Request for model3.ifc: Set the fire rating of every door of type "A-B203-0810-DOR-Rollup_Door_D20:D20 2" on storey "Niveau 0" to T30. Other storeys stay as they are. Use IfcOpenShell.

First a look at what the model holds.

```python
import ifcopenshell
import ifcopenshell.util.element

model = ifcopenshell.open("model3.ifc")
print(model.schema)
storey = next(s for s in model.by_type("IfcBuildingStorey") if s.Name == "Niveau 0")
doors = [e for e in ifcopenshell.util.element.get_decomposition(storey) if e.is_a("IfcDoor")]
seen = {}
for e in doors:
    element_type = ifcopenshell.util.element.get_type(e)
    key = (element_type.Name if element_type != e and element_type else None, ifcopenshell.util.element.get_pset(e, "Pset_DoorCommon", "FireRating"))
    seen[key] = seen.get(key, 0) + 1
for (name, value), count in sorted(seen.items(), key=str):
    print(count, "x", name, "|", value)
```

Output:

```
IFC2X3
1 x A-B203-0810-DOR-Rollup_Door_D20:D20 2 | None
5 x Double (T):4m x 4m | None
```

```python
import ifcopenshell
import ifcopenshell.api.pset
import ifcopenshell.util.element

model = ifcopenshell.open("model3.ifc")

storey = next(s for s in model.by_type("IfcBuildingStorey") if s.Name == "Niveau 0")
doors = [e for e in ifcopenshell.util.element.get_decomposition(storey) if e.is_a("IfcDoor")]

count = 0
for e in doors:
    element_type = ifcopenshell.util.element.get_type(e)
    if element_type in (None, e) or element_type.Name != "A-B203-0810-DOR-Rollup_Door_D20:D20 2":
        continue
    # add_pset returns the element's existing set when there is one.
    pset = ifcopenshell.api.pset.add_pset(model, product=e, name="Pset_DoorCommon")
    ifcopenshell.api.pset.edit_pset(model, pset=pset, properties={"FireRating": "T30"})
    count += 1

print(count, "doors updated")

model.write("model3_edited.ifc")
```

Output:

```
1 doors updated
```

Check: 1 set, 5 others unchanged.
